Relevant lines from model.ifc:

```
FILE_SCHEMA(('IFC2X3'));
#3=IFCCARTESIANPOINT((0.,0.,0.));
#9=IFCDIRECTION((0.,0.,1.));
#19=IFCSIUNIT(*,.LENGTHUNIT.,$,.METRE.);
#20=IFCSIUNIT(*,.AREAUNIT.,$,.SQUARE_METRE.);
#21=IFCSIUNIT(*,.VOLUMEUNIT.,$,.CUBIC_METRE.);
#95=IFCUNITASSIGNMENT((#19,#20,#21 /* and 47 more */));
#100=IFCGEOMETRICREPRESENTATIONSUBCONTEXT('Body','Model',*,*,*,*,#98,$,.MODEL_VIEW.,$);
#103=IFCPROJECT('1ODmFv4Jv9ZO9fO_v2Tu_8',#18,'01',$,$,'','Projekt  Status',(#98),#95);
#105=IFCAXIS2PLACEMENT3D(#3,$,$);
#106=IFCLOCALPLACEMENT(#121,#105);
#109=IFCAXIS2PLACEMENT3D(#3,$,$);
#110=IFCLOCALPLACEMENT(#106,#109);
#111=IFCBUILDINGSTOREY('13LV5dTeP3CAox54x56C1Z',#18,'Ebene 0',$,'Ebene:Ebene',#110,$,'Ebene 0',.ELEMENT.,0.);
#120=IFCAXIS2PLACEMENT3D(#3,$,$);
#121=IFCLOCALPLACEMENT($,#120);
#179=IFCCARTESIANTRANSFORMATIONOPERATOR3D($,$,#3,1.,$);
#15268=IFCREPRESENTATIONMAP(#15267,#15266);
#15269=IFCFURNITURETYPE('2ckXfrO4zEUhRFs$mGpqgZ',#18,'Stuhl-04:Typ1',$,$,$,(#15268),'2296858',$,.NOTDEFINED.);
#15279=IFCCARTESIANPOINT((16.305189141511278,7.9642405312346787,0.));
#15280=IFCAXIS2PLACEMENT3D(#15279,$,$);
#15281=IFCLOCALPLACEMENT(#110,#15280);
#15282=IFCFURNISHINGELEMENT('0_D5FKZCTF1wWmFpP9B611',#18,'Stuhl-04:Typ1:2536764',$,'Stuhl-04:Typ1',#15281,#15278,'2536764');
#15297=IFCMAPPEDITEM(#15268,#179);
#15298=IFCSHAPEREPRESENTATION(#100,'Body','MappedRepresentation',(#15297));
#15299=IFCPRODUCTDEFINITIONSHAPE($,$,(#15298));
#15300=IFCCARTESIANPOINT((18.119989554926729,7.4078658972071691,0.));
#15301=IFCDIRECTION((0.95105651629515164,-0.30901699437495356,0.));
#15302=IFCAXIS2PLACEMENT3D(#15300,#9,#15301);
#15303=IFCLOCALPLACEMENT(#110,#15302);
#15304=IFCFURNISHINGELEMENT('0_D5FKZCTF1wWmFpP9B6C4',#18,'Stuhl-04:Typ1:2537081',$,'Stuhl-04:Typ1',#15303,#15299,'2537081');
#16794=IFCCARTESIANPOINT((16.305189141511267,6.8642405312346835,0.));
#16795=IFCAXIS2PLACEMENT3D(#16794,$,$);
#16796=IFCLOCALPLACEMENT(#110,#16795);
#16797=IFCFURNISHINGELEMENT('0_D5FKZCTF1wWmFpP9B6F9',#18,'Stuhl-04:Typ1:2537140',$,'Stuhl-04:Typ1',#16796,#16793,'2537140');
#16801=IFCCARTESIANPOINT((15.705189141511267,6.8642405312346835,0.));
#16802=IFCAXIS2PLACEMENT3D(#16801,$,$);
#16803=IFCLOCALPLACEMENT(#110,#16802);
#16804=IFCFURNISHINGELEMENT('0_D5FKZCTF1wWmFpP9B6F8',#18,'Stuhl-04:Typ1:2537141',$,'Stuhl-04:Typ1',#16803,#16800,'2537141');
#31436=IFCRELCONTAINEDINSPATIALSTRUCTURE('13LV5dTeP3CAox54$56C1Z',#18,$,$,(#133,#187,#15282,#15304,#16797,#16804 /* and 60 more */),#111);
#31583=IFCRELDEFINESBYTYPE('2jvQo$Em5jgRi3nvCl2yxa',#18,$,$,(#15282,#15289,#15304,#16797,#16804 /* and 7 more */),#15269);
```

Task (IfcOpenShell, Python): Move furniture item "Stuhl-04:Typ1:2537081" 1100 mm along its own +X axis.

```python
import ifcopenshell
import ifcopenshell.api.geometry
import ifcopenshell.util.placement

model = ifcopenshell.open("model.ifc")

item = model.by_guid("0_D5FKZCTF1wWmFpP9B6C4")
matrix = ifcopenshell.util.placement.get_local_placement(item.ObjectPlacement)
matrix[:3, 3] += matrix[:3, 0] * 1.1
ifcopenshell.api.geometry.edit_object_placement(model, product=item, matrix=matrix, is_si=False)

print(ifcopenshell.util.placement.get_local_placement(item.ObjectPlacement).round(3) + 0.0)

model.write("model-out.ifc")
```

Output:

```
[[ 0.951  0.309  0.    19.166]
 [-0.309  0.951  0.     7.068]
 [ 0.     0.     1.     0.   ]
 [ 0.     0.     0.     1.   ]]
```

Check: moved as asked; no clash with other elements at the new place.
